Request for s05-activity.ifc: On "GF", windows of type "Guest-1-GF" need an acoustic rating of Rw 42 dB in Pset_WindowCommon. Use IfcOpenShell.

First a look at what the model holds.

```python
import ifcopenshell
import ifcopenshell.util.element

model = ifcopenshell.open("s05-activity.ifc")
print(model.schema)
storey = next(s for s in model.by_type("IfcBuildingStorey") if s.Name == "GF")
windows = [e for e in ifcopenshell.util.element.get_decomposition(storey) if e.is_a("IfcWindow")]
seen = {}
for e in windows:
    element_type = ifcopenshell.util.element.get_type(e)
    key = (element_type.Name if element_type != e and element_type else None, ifcopenshell.util.element.get_pset(e, "Pset_WindowCommon", "AcousticRating"))
    seen[key] = seen.get(key, 0) + 1
for (name, value), count in sorted(seen.items(), key=str):
    print(count, "x", name, "|", value)
```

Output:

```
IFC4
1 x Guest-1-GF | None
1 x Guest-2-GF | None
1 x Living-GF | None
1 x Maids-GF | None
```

```python
import ifcopenshell
import ifcopenshell.api.pset
import ifcopenshell.util.element

model = ifcopenshell.open("s05-activity.ifc")

storey = next(s for s in model.by_type("IfcBuildingStorey") if s.Name == "GF")
windows = [e for e in ifcopenshell.util.element.get_decomposition(storey) if e.is_a("IfcWindow")]

count = 0
for e in windows:
    element_type = ifcopenshell.util.element.get_type(e)
    if element_type in (None, e) or element_type.Name != "Guest-1-GF":
        continue
    # add_pset returns the element's existing set when there is one.
    pset = ifcopenshell.api.pset.add_pset(model, product=e, name="Pset_WindowCommon")
    ifcopenshell.api.pset.edit_pset(model, pset=pset, properties={"AcousticRating": "Rw 42 dB"})
    count += 1

print(count, "windows updated")

model.write("s05-activity-out.ifc")
```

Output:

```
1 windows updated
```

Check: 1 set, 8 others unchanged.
